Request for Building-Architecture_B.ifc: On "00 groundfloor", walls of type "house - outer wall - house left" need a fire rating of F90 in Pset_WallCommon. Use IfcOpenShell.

First a look at what the model holds.

```python
import ifcopenshell
import ifcopenshell.util.element

model = ifcopenshell.open("Building-Architecture_B.ifc")
print(model.schema)
storey = next(s for s in model.by_type("IfcBuildingStorey") if s.Name == "00 groundfloor")
walls = [e for e in ifcopenshell.util.element.get_decomposition(storey) if e.is_a("IfcWall")]
seen = {}
for e in walls:
    element_type = ifcopenshell.util.element.get_type(e)
    key = (element_type.Name if element_type != e and element_type else None, ifcopenshell.util.element.get_pset(e, "Pset_WallCommon", "FireRating"))
    seen[key] = seen.get(key, 0) + 1
for (name, value), count in sorted(seen.items(), key=str):
    print(count, "x", name, "|", value)
```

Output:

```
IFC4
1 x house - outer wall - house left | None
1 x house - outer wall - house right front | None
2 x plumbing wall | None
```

```python
import ifcopenshell
import ifcopenshell.api.pset
import ifcopenshell.util.element

model = ifcopenshell.open("Building-Architecture_B.ifc")

storey = next(s for s in model.by_type("IfcBuildingStorey") if s.Name == "00 groundfloor")
walls = [e for e in ifcopenshell.util.element.get_decomposition(storey) if e.is_a("IfcWall")]

count = 0
for e in walls:
    element_type = ifcopenshell.util.element.get_type(e)
    if element_type in (None, e) or element_type.Name != "house - outer wall - house left":
        continue
    # add_pset returns the element's existing set when there is one.
    pset = ifcopenshell.api.pset.add_pset(model, product=e, name="Pset_WallCommon")
    ifcopenshell.api.pset.edit_pset(model, pset=pset, properties={"FireRating": "F90"})
    count += 1

print(count, "walls updated")

model.write("Building-Architecture_B_edited.ifc")
```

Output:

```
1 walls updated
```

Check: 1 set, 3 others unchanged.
